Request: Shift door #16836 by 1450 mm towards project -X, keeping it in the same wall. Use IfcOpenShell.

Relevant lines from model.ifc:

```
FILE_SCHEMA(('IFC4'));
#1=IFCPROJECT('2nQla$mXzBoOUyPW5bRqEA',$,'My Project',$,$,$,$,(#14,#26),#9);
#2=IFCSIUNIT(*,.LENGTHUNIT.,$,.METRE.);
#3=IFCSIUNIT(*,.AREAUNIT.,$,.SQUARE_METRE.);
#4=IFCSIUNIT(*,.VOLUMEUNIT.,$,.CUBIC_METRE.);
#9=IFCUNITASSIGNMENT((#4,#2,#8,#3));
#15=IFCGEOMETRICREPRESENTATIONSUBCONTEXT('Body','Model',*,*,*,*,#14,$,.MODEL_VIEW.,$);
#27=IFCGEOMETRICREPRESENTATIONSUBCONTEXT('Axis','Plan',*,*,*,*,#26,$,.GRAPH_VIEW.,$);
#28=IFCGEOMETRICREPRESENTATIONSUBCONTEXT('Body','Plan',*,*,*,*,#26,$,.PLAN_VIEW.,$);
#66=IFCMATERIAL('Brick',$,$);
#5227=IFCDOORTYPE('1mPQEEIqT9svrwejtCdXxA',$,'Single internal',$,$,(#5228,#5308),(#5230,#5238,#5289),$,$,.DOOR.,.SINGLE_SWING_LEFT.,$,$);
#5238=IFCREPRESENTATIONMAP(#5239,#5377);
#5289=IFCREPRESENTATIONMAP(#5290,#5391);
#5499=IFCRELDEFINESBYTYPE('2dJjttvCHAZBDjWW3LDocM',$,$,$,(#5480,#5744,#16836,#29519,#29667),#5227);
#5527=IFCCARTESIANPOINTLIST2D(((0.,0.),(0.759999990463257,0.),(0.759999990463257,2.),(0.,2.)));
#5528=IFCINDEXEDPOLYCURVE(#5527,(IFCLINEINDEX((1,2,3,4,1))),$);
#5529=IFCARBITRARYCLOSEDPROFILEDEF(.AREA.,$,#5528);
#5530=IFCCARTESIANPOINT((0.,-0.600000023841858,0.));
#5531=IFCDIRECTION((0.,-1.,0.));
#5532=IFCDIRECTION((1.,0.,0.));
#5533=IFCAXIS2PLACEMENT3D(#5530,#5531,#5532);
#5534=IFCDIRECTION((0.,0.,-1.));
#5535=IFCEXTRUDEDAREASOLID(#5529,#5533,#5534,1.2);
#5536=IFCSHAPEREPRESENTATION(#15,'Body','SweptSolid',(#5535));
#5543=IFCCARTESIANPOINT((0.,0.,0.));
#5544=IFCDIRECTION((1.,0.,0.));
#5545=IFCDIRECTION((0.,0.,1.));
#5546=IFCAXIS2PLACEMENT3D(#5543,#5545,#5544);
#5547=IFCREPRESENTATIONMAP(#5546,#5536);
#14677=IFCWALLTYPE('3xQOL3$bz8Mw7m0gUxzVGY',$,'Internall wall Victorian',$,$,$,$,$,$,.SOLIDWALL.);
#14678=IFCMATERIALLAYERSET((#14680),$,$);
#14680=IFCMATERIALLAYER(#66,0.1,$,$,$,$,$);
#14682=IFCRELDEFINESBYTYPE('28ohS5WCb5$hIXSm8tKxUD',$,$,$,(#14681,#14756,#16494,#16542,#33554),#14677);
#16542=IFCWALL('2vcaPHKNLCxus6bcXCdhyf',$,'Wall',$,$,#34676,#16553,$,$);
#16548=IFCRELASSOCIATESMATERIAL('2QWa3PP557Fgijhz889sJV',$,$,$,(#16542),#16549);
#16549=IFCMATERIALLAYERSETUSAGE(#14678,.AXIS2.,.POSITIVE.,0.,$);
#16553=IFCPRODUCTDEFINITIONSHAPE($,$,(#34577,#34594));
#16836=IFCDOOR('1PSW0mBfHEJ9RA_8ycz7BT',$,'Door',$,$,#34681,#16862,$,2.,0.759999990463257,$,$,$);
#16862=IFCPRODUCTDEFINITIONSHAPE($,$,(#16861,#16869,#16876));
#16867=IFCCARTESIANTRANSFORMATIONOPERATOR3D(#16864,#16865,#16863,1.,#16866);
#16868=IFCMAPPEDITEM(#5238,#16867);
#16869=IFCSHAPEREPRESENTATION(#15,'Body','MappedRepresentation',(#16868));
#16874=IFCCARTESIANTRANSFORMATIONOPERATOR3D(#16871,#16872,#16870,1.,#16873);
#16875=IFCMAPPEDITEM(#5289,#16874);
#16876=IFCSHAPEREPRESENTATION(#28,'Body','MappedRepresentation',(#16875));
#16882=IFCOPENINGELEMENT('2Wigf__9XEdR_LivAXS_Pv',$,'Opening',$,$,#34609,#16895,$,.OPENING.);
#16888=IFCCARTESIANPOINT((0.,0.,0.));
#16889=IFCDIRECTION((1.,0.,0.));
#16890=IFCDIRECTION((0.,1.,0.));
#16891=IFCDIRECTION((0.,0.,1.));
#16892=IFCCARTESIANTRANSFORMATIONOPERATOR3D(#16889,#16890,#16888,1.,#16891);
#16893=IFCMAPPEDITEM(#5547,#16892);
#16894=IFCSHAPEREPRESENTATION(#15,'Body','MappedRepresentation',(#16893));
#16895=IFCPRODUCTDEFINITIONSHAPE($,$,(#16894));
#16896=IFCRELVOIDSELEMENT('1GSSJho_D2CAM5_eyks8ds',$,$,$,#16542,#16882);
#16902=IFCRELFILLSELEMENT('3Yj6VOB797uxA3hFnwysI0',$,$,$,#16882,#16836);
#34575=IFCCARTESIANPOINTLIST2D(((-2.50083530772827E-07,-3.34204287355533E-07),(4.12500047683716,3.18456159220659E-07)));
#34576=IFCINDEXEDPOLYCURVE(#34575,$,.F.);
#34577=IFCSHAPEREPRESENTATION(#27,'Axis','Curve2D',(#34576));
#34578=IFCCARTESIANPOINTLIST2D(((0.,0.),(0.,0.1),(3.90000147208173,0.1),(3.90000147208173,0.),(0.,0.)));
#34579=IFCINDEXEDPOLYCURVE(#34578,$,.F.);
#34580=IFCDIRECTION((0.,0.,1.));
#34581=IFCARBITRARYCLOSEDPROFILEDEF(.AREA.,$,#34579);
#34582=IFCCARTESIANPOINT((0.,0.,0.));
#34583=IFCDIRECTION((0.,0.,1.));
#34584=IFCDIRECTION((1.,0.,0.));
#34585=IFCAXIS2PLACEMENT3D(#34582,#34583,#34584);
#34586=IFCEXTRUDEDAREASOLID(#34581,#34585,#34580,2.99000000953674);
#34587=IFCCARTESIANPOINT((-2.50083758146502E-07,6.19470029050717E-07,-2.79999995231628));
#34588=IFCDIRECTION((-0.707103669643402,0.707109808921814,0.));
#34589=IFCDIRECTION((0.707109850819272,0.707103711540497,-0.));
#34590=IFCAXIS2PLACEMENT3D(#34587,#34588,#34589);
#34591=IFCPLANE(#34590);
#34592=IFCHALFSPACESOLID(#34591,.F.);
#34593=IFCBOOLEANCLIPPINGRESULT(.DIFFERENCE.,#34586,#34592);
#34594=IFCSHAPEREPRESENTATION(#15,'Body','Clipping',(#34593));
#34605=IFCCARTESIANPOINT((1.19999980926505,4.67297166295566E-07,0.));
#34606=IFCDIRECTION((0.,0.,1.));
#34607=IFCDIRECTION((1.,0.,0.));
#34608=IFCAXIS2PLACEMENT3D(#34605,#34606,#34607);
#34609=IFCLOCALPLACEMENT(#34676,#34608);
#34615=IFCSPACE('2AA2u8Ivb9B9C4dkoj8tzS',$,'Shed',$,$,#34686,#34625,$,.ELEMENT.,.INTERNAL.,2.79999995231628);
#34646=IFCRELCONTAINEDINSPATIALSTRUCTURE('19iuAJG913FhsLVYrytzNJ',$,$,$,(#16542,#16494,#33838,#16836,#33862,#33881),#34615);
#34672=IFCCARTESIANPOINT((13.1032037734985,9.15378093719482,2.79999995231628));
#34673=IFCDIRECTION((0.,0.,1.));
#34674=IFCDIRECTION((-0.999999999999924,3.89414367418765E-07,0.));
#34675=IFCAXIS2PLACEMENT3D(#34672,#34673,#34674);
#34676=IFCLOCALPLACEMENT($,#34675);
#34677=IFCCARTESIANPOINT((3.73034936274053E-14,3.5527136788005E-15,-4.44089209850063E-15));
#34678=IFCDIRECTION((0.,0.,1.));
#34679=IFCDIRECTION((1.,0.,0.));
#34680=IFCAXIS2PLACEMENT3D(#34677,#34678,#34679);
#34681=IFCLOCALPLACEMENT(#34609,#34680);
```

```python
import ifcopenshell
import ifcopenshell.api.geometry
import ifcopenshell.util.placement

model = ifcopenshell.open("model.ifc")

door = model.by_guid("1PSW0mBfHEJ9RA_8ycz7BT")
opening = door.FillsVoids[0].RelatingOpeningElement
wall = opening.VoidsElements[0].RelatingBuildingElement

wall_matrix = ifcopenshell.util.placement.get_local_placement(wall.ObjectPlacement)
shift = wall_matrix[:3, 0] * 1.45
before = ifcopenshell.util.placement.get_local_placement(door.ObjectPlacement)[:3, 3].copy()

# The door is placed relative to its opening, so it follows when the opening moves.
matrix = ifcopenshell.util.placement.get_local_placement(opening.ObjectPlacement)
matrix[:3, 3] += shift
ifcopenshell.api.geometry.edit_object_placement(
    model, product=opening, matrix=matrix, is_si=False, should_transform_children=True
)

after = ifcopenshell.util.placement.get_local_placement(door.ObjectPlacement)[:3, 3]
print("door moved by", (after - before).round(3) + 0.0)

model.write("model_v2.ifc")
```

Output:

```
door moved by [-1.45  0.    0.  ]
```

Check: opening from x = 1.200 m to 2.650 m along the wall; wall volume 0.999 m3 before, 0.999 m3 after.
